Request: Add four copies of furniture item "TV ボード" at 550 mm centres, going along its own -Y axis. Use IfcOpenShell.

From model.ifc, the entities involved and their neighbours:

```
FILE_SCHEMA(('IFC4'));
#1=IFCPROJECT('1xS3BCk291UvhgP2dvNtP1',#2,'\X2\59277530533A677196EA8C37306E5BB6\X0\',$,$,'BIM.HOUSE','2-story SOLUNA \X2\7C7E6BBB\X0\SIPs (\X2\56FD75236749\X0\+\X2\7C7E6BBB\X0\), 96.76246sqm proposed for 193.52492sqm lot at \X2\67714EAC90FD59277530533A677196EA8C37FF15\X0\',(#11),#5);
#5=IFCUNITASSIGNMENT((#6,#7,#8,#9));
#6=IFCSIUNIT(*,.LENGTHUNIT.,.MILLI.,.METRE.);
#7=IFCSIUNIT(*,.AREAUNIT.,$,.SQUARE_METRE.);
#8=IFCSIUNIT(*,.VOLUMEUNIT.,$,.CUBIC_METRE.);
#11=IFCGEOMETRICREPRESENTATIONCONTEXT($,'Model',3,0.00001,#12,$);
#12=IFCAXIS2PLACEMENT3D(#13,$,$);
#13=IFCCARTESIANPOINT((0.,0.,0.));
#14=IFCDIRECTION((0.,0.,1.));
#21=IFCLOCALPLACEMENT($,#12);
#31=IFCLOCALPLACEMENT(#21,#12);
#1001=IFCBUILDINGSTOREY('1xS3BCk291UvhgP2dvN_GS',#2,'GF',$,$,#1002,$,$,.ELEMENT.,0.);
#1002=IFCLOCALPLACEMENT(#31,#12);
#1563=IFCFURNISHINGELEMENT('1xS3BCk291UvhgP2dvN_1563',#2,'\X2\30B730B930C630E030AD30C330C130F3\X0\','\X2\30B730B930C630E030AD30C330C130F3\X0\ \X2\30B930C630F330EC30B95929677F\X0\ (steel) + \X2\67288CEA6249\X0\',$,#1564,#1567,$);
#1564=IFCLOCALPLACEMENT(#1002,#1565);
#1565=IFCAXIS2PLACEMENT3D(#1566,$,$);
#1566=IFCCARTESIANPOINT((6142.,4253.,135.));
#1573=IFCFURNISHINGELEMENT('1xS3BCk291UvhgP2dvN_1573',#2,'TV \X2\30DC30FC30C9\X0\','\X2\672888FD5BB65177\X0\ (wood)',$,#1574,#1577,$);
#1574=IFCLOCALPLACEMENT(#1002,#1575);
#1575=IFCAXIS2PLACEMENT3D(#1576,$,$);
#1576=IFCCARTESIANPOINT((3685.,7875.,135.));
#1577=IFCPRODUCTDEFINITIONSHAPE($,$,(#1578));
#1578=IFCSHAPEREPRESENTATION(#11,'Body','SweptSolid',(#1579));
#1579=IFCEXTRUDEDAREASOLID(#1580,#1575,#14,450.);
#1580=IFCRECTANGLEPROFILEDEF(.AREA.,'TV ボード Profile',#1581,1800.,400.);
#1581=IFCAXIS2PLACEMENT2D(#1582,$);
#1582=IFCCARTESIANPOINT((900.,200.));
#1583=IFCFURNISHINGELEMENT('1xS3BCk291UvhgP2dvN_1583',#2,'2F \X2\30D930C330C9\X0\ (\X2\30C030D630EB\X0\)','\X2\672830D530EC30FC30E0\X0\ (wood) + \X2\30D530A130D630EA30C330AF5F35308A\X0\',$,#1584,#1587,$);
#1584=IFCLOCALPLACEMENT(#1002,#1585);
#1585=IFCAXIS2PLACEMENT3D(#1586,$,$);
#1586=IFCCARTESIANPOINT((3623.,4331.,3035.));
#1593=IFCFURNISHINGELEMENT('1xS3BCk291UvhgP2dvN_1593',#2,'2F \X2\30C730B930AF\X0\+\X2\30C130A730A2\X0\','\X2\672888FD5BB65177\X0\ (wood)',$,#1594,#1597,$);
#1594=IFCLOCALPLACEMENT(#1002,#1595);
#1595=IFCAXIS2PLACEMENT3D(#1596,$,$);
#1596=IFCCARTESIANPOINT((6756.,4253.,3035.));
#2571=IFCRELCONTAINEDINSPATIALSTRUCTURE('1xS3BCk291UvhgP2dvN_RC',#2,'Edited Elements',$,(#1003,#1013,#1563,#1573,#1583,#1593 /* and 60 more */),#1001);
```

```python
import ifcopenshell
import ifcopenshell.api.geometry
import ifcopenshell.api.root
import ifcopenshell.util.element
import ifcopenshell.util.placement

model = ifcopenshell.open("model.ifc")


def reuse_history(source, copy):
    """copy_class also copies each property set's owner history, people and application; keep the originals."""
    for rel in copy.IsDefinedBy:
        if rel.is_a("IfcRelDefinesByProperties") and (history := rel.RelatingPropertyDefinition.OwnerHistory):
            rel.RelatingPropertyDefinition.OwnerHistory = source.OwnerHistory
            ifcopenshell.util.element.remove_deep2(model, history)


source = model.by_id(1573)
base = ifcopenshell.util.placement.get_local_placement(source.ObjectPlacement)
step = -base[:3, 1] * 550.0

for i in range(1, 5):
    copy = ifcopenshell.api.root.copy_class(model, product=source)
    copy.Representation = ifcopenshell.util.element.copy_deep(
        model, source.Representation, exclude=["IfcGeometricRepresentationContext", "IfcRepresentationMap"]
    )
    reuse_history(source, copy)
    matrix = base.copy()
    matrix[:3, 3] += i * step
    print("added at", matrix[:3, 3].round(3) + 0.0)
    ifcopenshell.api.geometry.edit_object_placement(model, product=copy, matrix=matrix, is_si=False)

model.write("model_edited.ifc")
```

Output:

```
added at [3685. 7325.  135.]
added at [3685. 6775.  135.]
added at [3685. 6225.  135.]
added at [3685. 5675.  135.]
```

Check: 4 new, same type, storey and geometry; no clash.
